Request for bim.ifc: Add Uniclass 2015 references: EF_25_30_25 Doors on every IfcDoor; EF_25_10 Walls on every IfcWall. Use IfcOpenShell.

First a look at what the model holds.

```python
import ifcopenshell

model = ifcopenshell.open("bim.ifc")
print(model.schema)
print("classifications:", [c.Name for c in model.by_type("IfcClassification")])
for ifc_class in ("IfcDoor", "IfcRoof", "IfcStair", "IfcWall", "IfcWindow"):
    print(ifc_class, len(model.by_type(ifc_class)))
```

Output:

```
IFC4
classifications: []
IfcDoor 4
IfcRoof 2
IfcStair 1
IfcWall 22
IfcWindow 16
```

```python
import ifcopenshell
import ifcopenshell.api.classification

model = ifcopenshell.open("bim.ifc")

system = ifcopenshell.api.classification.add_classification(model, classification="Uniclass 2015")

codes = {
    "IfcDoor": ("EF_25_30_25", "Doors"),
    "IfcWall": ("EF_25_10", "Walls"),
}
for ifc_class, (code, name) in codes.items():
    products = model.by_type(ifc_class)
    ifcopenshell.api.classification.add_reference(
        model, products=products, classification=system, identification=code, name=name
    )
    print(code, len(products))

model.write("bim_edited.ifc")
```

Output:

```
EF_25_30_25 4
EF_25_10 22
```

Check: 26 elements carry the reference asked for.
